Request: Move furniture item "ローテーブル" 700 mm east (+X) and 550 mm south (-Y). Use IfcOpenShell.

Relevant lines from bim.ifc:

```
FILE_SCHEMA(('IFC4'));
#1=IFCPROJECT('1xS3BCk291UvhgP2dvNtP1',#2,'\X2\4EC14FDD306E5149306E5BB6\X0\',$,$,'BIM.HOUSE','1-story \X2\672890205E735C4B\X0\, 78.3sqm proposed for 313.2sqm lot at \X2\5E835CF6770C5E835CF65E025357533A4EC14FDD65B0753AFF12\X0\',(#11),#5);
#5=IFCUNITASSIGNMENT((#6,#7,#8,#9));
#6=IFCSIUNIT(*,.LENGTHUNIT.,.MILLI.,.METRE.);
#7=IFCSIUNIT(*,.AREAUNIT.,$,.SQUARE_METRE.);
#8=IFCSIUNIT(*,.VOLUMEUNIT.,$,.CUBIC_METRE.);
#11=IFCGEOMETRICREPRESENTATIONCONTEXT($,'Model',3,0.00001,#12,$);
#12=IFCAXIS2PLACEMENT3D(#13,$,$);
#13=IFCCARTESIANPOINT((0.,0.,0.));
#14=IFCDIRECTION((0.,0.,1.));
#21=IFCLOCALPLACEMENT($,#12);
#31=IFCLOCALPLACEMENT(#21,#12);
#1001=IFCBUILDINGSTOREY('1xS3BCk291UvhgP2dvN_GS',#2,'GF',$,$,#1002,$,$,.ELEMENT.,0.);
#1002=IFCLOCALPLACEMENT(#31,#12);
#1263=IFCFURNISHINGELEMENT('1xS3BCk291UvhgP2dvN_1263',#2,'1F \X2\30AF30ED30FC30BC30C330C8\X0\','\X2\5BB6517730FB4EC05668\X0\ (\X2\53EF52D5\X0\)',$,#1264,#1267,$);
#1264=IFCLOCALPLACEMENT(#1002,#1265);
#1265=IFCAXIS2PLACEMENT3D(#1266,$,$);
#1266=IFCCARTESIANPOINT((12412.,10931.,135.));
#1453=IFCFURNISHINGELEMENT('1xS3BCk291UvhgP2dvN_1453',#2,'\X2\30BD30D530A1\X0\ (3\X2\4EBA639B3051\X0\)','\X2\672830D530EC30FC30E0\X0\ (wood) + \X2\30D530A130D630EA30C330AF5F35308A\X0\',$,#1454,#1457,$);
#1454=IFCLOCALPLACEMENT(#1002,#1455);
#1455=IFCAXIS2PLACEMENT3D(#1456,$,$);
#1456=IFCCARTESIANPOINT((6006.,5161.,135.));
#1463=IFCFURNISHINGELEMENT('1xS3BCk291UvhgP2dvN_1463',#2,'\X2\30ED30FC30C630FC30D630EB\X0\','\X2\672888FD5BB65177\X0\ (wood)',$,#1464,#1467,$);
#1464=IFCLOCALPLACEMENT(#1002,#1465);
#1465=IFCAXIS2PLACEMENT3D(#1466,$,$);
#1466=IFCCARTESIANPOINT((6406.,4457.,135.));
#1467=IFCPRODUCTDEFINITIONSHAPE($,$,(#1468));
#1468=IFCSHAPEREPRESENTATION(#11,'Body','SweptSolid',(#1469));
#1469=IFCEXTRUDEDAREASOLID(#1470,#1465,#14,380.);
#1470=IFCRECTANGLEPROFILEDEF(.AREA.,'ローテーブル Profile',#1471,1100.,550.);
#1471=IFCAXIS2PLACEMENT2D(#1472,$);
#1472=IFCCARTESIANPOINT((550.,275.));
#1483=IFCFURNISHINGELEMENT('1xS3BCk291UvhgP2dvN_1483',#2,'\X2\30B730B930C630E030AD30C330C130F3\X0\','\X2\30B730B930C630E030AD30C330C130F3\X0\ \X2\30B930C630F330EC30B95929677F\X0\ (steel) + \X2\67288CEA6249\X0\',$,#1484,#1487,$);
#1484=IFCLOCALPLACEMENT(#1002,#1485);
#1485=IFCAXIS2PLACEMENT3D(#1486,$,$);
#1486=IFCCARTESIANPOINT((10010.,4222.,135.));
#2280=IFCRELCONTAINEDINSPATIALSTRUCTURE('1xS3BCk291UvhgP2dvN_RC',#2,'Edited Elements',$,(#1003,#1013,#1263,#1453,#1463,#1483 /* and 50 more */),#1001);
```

```python
import ifcopenshell
import ifcopenshell.api.geometry
import ifcopenshell.util.placement

model = ifcopenshell.open("bim.ifc")

item = model.by_guid("1xS3BCk291UvhgP2dvN_1463")
matrix = ifcopenshell.util.placement.get_local_placement(item.ObjectPlacement)
matrix[0, 3] += 700.0
matrix[1, 3] -= 550.0
ifcopenshell.api.geometry.edit_object_placement(model, product=item, matrix=matrix, is_si=False)

print(ifcopenshell.util.placement.get_local_placement(item.ObjectPlacement).round(3) + 0.0)

model.write("bim-out.ifc")
```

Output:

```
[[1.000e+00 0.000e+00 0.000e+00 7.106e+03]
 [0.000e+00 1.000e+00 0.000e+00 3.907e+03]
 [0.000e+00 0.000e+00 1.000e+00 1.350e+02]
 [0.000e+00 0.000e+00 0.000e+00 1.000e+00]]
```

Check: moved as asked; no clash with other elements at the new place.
